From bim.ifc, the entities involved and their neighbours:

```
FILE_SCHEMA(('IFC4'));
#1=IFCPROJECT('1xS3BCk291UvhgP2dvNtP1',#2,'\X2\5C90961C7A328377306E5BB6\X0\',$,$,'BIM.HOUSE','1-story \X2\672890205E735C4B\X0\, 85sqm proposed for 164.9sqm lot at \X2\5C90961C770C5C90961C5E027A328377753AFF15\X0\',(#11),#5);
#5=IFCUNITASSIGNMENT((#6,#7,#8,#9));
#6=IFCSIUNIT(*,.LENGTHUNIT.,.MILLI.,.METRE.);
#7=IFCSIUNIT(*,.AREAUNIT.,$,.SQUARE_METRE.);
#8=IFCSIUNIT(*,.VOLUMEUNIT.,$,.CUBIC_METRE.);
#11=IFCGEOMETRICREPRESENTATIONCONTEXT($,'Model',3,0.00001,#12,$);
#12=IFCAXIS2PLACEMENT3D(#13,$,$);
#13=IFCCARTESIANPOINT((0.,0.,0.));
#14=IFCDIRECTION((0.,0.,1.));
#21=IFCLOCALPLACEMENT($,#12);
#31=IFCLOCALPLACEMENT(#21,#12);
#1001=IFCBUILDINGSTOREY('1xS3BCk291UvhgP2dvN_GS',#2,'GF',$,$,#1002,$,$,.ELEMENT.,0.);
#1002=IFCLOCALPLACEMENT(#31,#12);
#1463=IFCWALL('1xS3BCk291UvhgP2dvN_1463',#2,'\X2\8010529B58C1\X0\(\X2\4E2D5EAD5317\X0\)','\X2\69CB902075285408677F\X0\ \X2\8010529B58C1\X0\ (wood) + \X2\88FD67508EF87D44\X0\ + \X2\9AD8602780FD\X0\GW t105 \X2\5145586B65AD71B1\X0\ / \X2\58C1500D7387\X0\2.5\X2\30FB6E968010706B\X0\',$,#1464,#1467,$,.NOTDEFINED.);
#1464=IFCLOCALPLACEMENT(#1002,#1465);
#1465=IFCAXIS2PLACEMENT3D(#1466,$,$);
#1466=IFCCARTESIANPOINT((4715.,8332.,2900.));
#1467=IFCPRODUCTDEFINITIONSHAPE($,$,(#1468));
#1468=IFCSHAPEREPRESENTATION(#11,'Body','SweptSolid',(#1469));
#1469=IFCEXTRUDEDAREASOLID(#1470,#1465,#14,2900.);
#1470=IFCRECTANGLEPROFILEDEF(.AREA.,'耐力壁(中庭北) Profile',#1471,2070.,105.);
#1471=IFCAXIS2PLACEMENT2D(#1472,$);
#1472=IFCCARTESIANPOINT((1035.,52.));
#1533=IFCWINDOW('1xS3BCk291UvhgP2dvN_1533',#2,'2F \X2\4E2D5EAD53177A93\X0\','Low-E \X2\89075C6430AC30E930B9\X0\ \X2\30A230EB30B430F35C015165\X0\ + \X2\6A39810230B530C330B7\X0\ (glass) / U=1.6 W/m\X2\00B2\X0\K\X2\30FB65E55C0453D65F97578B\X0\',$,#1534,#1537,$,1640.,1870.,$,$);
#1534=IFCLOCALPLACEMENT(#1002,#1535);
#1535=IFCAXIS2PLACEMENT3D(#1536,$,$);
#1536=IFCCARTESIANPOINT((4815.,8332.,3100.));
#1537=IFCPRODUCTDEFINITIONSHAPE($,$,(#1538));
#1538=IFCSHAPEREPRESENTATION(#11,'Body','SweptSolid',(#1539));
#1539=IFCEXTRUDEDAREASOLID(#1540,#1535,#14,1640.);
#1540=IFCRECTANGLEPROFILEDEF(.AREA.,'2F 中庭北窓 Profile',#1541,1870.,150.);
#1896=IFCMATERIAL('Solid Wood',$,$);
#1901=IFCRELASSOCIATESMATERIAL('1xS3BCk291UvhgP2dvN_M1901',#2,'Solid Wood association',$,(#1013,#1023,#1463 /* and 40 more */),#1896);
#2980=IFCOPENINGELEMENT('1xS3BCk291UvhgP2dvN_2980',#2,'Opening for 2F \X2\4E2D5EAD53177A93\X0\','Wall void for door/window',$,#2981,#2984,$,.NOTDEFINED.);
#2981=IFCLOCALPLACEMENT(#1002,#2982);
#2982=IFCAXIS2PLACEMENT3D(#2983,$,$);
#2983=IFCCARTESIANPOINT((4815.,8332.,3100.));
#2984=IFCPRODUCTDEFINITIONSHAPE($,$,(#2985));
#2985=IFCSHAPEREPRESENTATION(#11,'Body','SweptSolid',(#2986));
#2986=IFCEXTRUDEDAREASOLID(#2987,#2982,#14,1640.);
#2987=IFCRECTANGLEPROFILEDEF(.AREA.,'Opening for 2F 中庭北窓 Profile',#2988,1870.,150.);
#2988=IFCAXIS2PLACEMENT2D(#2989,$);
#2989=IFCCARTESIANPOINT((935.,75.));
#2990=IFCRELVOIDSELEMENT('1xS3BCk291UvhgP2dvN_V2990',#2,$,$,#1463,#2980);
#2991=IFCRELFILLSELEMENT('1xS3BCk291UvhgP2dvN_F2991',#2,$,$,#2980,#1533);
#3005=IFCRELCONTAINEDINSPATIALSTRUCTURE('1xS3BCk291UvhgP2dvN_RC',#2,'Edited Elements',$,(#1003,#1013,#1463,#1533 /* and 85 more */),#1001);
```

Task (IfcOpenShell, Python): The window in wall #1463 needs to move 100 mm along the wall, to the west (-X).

```python
import ifcopenshell
import ifcopenshell.api.geometry
import ifcopenshell.util.placement
import ifcopenshell.util.unit

model = ifcopenshell.open("bim.ifc")
unit_scale = ifcopenshell.util.unit.calculate_unit_scale(model)

window = model.by_guid("1xS3BCk291UvhgP2dvN_1533")
opening = window.FillsVoids[0].RelatingOpeningElement
wall = opening.VoidsElements[0].RelatingBuildingElement

wall_matrix = ifcopenshell.util.placement.get_local_placement(wall.ObjectPlacement)
shift = wall_matrix[:3, 0] * -0.1 / unit_scale
before = ifcopenshell.util.placement.get_local_placement(window.ObjectPlacement)[:3, 3].copy()

# The window is not placed relative to its opening, so move both.
for product in (opening, window):
    matrix = ifcopenshell.util.placement.get_local_placement(product.ObjectPlacement)
    matrix[:3, 3] += shift
    ifcopenshell.api.geometry.edit_object_placement(model, product=product, matrix=matrix, is_si=False)

after = ifcopenshell.util.placement.get_local_placement(window.ObjectPlacement)[:3, 3]
print("window moved by", (after - before).round(3) + 0.0)

model.write("bim-out.ifc")
```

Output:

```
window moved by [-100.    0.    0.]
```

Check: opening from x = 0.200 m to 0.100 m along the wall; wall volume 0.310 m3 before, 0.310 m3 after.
